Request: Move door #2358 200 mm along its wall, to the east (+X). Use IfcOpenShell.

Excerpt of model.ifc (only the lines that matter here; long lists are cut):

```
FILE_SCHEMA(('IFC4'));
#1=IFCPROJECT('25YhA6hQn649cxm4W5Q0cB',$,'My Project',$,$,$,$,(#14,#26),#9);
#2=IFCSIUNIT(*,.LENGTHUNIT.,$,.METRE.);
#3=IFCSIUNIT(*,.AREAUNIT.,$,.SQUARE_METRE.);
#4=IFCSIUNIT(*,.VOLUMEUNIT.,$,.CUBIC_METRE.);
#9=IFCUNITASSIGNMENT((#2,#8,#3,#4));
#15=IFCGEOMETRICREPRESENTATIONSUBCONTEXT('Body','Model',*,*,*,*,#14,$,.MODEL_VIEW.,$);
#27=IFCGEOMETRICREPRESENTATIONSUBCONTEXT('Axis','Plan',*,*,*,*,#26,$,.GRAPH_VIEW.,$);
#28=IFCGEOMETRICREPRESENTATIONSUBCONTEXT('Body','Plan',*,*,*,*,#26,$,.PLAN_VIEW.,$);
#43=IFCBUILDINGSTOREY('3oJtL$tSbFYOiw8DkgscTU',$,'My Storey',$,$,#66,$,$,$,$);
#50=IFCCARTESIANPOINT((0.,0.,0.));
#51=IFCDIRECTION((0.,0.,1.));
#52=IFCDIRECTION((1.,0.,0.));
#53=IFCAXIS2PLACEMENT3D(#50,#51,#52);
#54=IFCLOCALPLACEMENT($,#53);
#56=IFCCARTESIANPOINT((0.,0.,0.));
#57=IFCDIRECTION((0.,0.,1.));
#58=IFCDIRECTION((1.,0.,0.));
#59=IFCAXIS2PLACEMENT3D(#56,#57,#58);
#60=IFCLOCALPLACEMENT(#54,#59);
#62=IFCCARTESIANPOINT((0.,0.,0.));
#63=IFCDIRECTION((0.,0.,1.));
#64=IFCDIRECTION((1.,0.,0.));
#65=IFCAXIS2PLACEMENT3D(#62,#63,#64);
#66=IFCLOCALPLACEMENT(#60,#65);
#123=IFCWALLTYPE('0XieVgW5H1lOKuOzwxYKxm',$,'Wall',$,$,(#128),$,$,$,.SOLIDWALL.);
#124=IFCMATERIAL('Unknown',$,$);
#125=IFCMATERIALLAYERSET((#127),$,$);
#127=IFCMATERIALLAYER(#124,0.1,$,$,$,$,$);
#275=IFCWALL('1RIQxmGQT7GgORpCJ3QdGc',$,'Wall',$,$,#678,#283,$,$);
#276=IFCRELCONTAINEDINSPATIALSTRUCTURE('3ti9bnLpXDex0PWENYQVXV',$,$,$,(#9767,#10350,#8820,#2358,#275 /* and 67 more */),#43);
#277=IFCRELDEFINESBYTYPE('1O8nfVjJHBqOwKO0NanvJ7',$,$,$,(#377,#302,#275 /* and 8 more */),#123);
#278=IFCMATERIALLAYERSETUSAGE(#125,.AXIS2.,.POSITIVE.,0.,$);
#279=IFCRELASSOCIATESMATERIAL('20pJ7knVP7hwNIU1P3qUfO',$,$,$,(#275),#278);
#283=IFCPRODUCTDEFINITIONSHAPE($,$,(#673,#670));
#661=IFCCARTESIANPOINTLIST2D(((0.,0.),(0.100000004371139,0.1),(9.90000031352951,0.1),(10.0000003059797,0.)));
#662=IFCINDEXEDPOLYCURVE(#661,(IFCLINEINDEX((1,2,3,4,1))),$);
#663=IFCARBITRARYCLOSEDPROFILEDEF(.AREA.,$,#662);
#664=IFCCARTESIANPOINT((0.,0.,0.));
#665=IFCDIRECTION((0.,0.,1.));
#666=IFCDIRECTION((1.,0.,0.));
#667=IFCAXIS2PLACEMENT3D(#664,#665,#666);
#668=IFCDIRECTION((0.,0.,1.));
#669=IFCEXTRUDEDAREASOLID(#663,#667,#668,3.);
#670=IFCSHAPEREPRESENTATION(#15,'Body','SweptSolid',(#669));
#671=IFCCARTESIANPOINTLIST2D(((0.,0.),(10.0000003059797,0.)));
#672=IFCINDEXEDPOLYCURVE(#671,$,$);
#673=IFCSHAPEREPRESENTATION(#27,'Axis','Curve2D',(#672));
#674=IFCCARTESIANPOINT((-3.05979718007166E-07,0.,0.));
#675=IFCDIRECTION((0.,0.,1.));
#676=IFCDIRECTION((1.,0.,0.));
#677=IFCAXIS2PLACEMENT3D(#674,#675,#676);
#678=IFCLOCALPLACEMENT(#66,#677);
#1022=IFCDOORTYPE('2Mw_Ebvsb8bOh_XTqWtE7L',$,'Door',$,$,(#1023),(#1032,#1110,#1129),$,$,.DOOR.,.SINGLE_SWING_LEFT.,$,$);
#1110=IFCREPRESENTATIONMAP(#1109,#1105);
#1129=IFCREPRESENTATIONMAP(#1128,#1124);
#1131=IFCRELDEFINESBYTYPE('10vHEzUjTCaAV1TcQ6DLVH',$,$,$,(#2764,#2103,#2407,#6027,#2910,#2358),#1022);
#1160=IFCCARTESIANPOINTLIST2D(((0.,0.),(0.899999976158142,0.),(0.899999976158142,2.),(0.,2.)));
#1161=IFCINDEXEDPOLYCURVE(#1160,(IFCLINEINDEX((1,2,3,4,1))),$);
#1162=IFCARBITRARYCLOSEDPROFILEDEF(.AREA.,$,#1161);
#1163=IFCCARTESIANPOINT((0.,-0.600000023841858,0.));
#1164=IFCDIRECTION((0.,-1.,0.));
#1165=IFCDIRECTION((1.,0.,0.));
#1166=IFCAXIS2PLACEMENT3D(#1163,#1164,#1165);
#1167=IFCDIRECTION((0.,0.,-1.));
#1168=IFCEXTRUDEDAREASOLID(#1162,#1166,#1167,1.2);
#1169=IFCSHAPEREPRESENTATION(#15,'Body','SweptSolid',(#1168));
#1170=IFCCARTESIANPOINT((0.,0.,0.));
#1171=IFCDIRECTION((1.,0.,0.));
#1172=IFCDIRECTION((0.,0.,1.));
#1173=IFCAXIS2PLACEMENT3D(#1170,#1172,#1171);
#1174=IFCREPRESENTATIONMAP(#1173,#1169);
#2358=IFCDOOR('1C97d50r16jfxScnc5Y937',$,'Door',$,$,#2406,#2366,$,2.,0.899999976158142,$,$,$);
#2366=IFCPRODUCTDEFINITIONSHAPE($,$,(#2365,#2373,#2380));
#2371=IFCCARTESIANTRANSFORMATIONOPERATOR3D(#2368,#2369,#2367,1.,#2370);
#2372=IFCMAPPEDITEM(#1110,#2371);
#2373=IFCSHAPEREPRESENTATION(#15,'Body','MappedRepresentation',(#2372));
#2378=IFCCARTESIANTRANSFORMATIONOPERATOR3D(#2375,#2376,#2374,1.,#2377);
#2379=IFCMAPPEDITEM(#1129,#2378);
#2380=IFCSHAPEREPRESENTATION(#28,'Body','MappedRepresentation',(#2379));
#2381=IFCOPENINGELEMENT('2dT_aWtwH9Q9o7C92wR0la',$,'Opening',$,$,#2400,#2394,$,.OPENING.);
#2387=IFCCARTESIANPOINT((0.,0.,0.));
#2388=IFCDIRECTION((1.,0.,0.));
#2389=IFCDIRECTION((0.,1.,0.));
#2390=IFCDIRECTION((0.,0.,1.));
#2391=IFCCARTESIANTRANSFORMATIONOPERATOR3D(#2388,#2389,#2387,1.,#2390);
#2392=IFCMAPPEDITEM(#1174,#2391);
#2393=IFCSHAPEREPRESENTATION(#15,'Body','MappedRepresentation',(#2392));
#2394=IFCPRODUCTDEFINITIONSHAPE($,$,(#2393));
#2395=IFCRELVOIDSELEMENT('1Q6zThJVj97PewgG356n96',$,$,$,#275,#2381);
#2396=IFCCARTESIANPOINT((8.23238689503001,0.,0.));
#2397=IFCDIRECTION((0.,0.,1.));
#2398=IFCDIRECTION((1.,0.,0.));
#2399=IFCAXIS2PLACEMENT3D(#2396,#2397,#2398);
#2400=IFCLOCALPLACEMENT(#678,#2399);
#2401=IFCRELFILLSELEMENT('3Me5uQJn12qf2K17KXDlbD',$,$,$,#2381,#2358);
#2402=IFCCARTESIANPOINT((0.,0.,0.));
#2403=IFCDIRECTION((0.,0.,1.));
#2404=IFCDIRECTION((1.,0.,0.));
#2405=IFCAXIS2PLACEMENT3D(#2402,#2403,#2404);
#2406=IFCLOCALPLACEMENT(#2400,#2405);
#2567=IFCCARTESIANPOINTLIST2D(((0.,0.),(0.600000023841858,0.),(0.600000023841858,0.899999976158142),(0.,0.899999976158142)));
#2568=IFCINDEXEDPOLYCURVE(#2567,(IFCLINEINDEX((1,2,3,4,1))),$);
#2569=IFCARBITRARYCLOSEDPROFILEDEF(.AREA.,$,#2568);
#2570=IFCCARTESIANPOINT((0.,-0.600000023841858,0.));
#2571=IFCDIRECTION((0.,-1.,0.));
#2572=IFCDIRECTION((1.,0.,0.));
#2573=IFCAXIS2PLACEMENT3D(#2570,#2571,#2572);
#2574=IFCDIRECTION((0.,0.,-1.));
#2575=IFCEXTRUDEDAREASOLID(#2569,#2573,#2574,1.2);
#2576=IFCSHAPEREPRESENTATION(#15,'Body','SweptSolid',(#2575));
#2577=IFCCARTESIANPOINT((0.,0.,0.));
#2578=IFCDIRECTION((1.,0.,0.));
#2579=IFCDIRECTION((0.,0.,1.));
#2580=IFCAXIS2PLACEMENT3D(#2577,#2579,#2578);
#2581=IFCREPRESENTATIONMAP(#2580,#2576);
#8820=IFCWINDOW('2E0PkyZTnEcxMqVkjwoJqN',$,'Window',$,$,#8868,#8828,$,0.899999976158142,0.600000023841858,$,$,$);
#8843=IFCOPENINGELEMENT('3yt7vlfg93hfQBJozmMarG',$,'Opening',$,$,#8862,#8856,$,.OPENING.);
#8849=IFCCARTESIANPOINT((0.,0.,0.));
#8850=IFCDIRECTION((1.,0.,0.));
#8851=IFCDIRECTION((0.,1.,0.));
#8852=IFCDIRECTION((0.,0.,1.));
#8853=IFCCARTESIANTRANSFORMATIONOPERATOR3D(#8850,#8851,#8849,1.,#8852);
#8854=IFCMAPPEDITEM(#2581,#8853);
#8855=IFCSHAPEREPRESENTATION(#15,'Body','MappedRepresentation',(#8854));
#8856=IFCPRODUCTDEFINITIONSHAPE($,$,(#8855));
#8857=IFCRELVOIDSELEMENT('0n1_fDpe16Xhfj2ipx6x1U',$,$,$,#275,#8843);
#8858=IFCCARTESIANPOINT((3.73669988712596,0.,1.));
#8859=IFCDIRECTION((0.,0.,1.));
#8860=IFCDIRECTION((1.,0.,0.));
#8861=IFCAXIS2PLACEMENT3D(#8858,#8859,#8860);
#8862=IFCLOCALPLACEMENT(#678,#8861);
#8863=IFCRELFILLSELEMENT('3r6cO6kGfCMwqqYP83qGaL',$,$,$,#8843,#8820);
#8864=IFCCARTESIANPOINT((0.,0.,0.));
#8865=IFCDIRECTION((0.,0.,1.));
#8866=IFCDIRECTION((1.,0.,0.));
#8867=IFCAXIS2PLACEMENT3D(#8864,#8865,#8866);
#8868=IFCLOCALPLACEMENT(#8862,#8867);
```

```python
import ifcopenshell
import ifcopenshell.api.geometry
import ifcopenshell.util.placement
import ifcopenshell.util.unit

model = ifcopenshell.open("model.ifc")
unit_scale = ifcopenshell.util.unit.calculate_unit_scale(model)

door = model.by_id(2358)
opening = door.FillsVoids[0].RelatingOpeningElement
wall = opening.VoidsElements[0].RelatingBuildingElement

wall_matrix = ifcopenshell.util.placement.get_local_placement(wall.ObjectPlacement)
shift = wall_matrix[:3, 0] * 0.2 / unit_scale
before = ifcopenshell.util.placement.get_local_placement(door.ObjectPlacement)[:3, 3].copy()

# The door is placed relative to its opening, so it follows when the opening moves.
matrix = ifcopenshell.util.placement.get_local_placement(opening.ObjectPlacement)
matrix[:3, 3] += shift
ifcopenshell.api.geometry.edit_object_placement(
    model, product=opening, matrix=matrix, is_si=False, should_transform_children=True
)

after = ifcopenshell.util.placement.get_local_placement(door.ObjectPlacement)[:3, 3]
print("door moved by", (after - before).round(3) + 0.0)

model.write("model_edited.ifc")
```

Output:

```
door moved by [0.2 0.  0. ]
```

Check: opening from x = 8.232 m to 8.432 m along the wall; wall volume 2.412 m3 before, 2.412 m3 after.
